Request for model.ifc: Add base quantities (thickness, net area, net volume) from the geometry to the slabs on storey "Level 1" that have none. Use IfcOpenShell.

First a look at what the model holds.

```python
import ifcopenshell
import ifcopenshell.util.element
import ifcopenshell.util.unit

model = ifcopenshell.open("model.ifc")
print(model.schema)
for unit_type in ("LENGTHUNIT", "AREAUNIT", "VOLUMEUNIT"):
    print(unit_type, ifcopenshell.util.unit.calculate_unit_scale(model, unit_type))
storey = next(s for s in model.by_type("IfcBuildingStorey") if s.Name == "Level 1")
slabs = [e for e in ifcopenshell.util.element.get_decomposition(storey) if e.is_a("IfcSlab")]
for e in sorted(slabs, key=lambda e: e.id()):
    print(e.id(), e.is_a(), e.Name, list(ifcopenshell.util.element.get_psets(e, qtos_only=True)), sep=" | ")
```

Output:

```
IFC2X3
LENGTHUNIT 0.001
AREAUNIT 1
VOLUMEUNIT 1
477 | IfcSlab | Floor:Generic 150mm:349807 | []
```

```python
import ifcopenshell
import ifcopenshell.api.pset
import ifcopenshell.geom
import ifcopenshell.util.element
import ifcopenshell.util.shape
import ifcopenshell.util.unit

model = ifcopenshell.open("model.ifc")
unit_scale = ifcopenshell.util.unit.calculate_unit_scale(model)
area_scale = ifcopenshell.util.unit.calculate_unit_scale(model, "AREAUNIT")
volume_scale = ifcopenshell.util.unit.calculate_unit_scale(model, "VOLUMEUNIT")
settings = ifcopenshell.geom.settings()

storey = next(s for s in model.by_type("IfcBuildingStorey") if s.Name == "Level 1")
slabs = [e for e in ifcopenshell.util.element.get_decomposition(storey) if e.is_a("IfcSlab")]

for e in sorted(slabs, key=lambda e: e.id()):
    if ifcopenshell.util.element.get_psets(e, qtos_only=True, should_inherit=False):
        continue
    # Geometry comes back in metres, in the element's own axes.
    shape = ifcopenshell.geom.create_shape(settings, e)
    values = {
        "Width": ifcopenshell.util.shape.get_z(shape.geometry) / unit_scale,
        "NetArea": ifcopenshell.util.shape.get_footprint_area(shape.geometry) / area_scale,
        "NetVolume": ifcopenshell.util.shape.get_volume(shape.geometry) / volume_scale,
    }
    qto = ifcopenshell.api.pset.add_qto(model, product=e, name="BaseQuantities")
    ifcopenshell.api.pset.edit_qto(model, qto=qto, properties=values)
    print(e.id(), {k: round(v, 3) for k, v in values.items()})

model.write("model_rev.ifc")
```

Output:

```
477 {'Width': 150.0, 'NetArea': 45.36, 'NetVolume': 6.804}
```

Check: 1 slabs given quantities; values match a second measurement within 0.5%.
